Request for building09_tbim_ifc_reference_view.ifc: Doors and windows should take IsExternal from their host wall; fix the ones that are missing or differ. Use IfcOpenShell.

First a look at what the model holds.

```python
import ifcopenshell
import ifcopenshell.util.element

model = ifcopenshell.open("building09_tbim_ifc_reference_view.ifc")
print(model.schema)
seen = {}
for e in model.by_type("IfcDoor") + model.by_type("IfcWindow"):
    if not e.FillsVoids:
        continue
    host = e.FillsVoids[0].RelatingOpeningElement.VoidsElements[0].RelatingBuildingElement
    own = ifcopenshell.util.element.get_pset(e, f"Pset_{e.is_a()[3:].removesuffix('StandardCase')}Common", "IsExternal")
    wall = ifcopenshell.util.element.get_pset(host, "Pset_WallCommon", "IsExternal")
    seen[e.is_a(), own, wall] = seen.get((e.is_a(), own, wall), 0) + 1
for (cls, own, wall), count in sorted(seen.items(), key=str):
    print(count, cls, "IsExternal:", own, "| host wall:", wall)
```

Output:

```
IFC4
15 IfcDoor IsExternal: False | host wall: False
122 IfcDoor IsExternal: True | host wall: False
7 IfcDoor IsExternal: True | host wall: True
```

```python
import ifcopenshell
import ifcopenshell.api.pset
import ifcopenshell.util.element

model = ifcopenshell.open("building09_tbim_ifc_reference_view.ifc")

count = 0
for ifc_class, pset_name in (("IfcDoor", "Pset_DoorCommon"), ("IfcWindow", "Pset_WindowCommon")):
    for e in model.by_type(ifc_class):
        if not e.FillsVoids:
            continue
        host = e.FillsVoids[0].RelatingOpeningElement.VoidsElements[0].RelatingBuildingElement
        external = ifcopenshell.util.element.get_pset(host, "Pset_WallCommon", "IsExternal")
        if external is None or ifcopenshell.util.element.get_pset(e, pset_name, "IsExternal") == external:
            continue
        pset = ifcopenshell.api.pset.add_pset(model, product=e, name=pset_name)
        ifcopenshell.api.pset.edit_pset(model, pset=pset, properties={"IsExternal": external})
        count += 1

print(count, "updated")

model.write("building09_tbim_ifc_reference_view_edited.ifc")
```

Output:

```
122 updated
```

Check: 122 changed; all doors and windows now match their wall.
